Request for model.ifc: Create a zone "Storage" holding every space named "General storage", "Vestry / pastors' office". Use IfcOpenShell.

First a look at what the model holds.

```python
import ifcopenshell

model = ifcopenshell.open("model.ifc")
print(model.schema)
seen = {}
for space in model.by_type("IfcSpace"):
    seen[space.LongName] = seen.get(space.LongName, 0) + 1
for name, count in sorted(seen.items(), key=str):
    print(count, "x", name)
print("zones:", [z.Name for z in model.by_type("IfcZone")][:20])
```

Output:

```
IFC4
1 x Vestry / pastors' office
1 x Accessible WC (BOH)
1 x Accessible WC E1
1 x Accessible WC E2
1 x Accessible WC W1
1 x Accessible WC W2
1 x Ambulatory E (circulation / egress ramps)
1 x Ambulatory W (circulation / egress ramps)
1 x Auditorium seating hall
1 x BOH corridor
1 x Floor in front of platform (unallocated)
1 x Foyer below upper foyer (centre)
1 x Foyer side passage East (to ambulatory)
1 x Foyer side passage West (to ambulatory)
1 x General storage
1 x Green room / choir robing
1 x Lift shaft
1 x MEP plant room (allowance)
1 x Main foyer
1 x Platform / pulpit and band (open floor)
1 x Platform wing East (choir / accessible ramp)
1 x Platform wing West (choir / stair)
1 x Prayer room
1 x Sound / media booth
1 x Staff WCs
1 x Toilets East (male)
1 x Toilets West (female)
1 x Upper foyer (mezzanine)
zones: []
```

```python
import ifcopenshell
import ifcopenshell.api.group
import ifcopenshell.api.root

model = ifcopenshell.open("model.ifc")

names = {"General storage", "Vestry / pastors' office"}
spaces = [s for s in model.by_type("IfcSpace") if s.LongName in names]

zone = ifcopenshell.api.root.create_entity(model, ifc_class="IfcZone", name="Storage")
ifcopenshell.api.group.assign_group(model, products=spaces, group=zone)
print(len(spaces), "spaces in", zone.Name)

model.write("model_edited.ifc")
```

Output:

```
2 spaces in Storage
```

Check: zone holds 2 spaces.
